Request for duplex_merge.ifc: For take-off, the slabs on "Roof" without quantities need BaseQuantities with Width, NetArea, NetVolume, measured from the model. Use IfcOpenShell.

First a look at what the model holds.

```python
import ifcopenshell
import ifcopenshell.util.element
import ifcopenshell.util.unit

model = ifcopenshell.open("duplex_merge.ifc")
print(model.schema)
for unit_type in ("LENGTHUNIT", "AREAUNIT", "VOLUMEUNIT"):
    print(unit_type, ifcopenshell.util.unit.calculate_unit_scale(model, unit_type))
storey = next(s for s in model.by_type("IfcBuildingStorey") if s.Name == "Roof")
slabs = [e for e in ifcopenshell.util.element.get_decomposition(storey) if e.is_a("IfcSlab")]
for e in sorted(slabs, key=lambda e: e.id()):
    print(e.id(), e.is_a(), e.Name, list(ifcopenshell.util.element.get_psets(e, qtos_only=True)), sep=" | ")
```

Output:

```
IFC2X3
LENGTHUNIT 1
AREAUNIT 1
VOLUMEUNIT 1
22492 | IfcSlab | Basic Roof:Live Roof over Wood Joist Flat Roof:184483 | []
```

```python
import ifcopenshell
import ifcopenshell.api.pset
import ifcopenshell.geom
import ifcopenshell.util.element
import ifcopenshell.util.shape
import ifcopenshell.util.unit

model = ifcopenshell.open("duplex_merge.ifc")
unit_scale = ifcopenshell.util.unit.calculate_unit_scale(model)
area_scale = ifcopenshell.util.unit.calculate_unit_scale(model, "AREAUNIT")
volume_scale = ifcopenshell.util.unit.calculate_unit_scale(model, "VOLUMEUNIT")
settings = ifcopenshell.geom.settings()

storey = next(s for s in model.by_type("IfcBuildingStorey") if s.Name == "Roof")
slabs = [e for e in ifcopenshell.util.element.get_decomposition(storey) if e.is_a("IfcSlab")]

for e in sorted(slabs, key=lambda e: e.id()):
    if ifcopenshell.util.element.get_psets(e, qtos_only=True, should_inherit=False):
        continue
    # Geometry comes back in metres, in the element's own axes.
    shape = ifcopenshell.geom.create_shape(settings, e)
    values = {
        "Width": ifcopenshell.util.shape.get_z(shape.geometry) / unit_scale,
        "NetArea": ifcopenshell.util.shape.get_footprint_area(shape.geometry) / area_scale,
        "NetVolume": ifcopenshell.util.shape.get_volume(shape.geometry) / volume_scale,
    }
    qto = ifcopenshell.api.pset.add_qto(model, product=e, name="BaseQuantities")
    ifcopenshell.api.pset.edit_qto(model, qto=qto, properties=values)
    print(e.id(), {k: round(v, 3) for k, v in values.items()})

model.write("duplex_merge-out.ifc")
```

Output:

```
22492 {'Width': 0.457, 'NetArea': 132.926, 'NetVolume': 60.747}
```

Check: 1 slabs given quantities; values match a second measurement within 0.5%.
